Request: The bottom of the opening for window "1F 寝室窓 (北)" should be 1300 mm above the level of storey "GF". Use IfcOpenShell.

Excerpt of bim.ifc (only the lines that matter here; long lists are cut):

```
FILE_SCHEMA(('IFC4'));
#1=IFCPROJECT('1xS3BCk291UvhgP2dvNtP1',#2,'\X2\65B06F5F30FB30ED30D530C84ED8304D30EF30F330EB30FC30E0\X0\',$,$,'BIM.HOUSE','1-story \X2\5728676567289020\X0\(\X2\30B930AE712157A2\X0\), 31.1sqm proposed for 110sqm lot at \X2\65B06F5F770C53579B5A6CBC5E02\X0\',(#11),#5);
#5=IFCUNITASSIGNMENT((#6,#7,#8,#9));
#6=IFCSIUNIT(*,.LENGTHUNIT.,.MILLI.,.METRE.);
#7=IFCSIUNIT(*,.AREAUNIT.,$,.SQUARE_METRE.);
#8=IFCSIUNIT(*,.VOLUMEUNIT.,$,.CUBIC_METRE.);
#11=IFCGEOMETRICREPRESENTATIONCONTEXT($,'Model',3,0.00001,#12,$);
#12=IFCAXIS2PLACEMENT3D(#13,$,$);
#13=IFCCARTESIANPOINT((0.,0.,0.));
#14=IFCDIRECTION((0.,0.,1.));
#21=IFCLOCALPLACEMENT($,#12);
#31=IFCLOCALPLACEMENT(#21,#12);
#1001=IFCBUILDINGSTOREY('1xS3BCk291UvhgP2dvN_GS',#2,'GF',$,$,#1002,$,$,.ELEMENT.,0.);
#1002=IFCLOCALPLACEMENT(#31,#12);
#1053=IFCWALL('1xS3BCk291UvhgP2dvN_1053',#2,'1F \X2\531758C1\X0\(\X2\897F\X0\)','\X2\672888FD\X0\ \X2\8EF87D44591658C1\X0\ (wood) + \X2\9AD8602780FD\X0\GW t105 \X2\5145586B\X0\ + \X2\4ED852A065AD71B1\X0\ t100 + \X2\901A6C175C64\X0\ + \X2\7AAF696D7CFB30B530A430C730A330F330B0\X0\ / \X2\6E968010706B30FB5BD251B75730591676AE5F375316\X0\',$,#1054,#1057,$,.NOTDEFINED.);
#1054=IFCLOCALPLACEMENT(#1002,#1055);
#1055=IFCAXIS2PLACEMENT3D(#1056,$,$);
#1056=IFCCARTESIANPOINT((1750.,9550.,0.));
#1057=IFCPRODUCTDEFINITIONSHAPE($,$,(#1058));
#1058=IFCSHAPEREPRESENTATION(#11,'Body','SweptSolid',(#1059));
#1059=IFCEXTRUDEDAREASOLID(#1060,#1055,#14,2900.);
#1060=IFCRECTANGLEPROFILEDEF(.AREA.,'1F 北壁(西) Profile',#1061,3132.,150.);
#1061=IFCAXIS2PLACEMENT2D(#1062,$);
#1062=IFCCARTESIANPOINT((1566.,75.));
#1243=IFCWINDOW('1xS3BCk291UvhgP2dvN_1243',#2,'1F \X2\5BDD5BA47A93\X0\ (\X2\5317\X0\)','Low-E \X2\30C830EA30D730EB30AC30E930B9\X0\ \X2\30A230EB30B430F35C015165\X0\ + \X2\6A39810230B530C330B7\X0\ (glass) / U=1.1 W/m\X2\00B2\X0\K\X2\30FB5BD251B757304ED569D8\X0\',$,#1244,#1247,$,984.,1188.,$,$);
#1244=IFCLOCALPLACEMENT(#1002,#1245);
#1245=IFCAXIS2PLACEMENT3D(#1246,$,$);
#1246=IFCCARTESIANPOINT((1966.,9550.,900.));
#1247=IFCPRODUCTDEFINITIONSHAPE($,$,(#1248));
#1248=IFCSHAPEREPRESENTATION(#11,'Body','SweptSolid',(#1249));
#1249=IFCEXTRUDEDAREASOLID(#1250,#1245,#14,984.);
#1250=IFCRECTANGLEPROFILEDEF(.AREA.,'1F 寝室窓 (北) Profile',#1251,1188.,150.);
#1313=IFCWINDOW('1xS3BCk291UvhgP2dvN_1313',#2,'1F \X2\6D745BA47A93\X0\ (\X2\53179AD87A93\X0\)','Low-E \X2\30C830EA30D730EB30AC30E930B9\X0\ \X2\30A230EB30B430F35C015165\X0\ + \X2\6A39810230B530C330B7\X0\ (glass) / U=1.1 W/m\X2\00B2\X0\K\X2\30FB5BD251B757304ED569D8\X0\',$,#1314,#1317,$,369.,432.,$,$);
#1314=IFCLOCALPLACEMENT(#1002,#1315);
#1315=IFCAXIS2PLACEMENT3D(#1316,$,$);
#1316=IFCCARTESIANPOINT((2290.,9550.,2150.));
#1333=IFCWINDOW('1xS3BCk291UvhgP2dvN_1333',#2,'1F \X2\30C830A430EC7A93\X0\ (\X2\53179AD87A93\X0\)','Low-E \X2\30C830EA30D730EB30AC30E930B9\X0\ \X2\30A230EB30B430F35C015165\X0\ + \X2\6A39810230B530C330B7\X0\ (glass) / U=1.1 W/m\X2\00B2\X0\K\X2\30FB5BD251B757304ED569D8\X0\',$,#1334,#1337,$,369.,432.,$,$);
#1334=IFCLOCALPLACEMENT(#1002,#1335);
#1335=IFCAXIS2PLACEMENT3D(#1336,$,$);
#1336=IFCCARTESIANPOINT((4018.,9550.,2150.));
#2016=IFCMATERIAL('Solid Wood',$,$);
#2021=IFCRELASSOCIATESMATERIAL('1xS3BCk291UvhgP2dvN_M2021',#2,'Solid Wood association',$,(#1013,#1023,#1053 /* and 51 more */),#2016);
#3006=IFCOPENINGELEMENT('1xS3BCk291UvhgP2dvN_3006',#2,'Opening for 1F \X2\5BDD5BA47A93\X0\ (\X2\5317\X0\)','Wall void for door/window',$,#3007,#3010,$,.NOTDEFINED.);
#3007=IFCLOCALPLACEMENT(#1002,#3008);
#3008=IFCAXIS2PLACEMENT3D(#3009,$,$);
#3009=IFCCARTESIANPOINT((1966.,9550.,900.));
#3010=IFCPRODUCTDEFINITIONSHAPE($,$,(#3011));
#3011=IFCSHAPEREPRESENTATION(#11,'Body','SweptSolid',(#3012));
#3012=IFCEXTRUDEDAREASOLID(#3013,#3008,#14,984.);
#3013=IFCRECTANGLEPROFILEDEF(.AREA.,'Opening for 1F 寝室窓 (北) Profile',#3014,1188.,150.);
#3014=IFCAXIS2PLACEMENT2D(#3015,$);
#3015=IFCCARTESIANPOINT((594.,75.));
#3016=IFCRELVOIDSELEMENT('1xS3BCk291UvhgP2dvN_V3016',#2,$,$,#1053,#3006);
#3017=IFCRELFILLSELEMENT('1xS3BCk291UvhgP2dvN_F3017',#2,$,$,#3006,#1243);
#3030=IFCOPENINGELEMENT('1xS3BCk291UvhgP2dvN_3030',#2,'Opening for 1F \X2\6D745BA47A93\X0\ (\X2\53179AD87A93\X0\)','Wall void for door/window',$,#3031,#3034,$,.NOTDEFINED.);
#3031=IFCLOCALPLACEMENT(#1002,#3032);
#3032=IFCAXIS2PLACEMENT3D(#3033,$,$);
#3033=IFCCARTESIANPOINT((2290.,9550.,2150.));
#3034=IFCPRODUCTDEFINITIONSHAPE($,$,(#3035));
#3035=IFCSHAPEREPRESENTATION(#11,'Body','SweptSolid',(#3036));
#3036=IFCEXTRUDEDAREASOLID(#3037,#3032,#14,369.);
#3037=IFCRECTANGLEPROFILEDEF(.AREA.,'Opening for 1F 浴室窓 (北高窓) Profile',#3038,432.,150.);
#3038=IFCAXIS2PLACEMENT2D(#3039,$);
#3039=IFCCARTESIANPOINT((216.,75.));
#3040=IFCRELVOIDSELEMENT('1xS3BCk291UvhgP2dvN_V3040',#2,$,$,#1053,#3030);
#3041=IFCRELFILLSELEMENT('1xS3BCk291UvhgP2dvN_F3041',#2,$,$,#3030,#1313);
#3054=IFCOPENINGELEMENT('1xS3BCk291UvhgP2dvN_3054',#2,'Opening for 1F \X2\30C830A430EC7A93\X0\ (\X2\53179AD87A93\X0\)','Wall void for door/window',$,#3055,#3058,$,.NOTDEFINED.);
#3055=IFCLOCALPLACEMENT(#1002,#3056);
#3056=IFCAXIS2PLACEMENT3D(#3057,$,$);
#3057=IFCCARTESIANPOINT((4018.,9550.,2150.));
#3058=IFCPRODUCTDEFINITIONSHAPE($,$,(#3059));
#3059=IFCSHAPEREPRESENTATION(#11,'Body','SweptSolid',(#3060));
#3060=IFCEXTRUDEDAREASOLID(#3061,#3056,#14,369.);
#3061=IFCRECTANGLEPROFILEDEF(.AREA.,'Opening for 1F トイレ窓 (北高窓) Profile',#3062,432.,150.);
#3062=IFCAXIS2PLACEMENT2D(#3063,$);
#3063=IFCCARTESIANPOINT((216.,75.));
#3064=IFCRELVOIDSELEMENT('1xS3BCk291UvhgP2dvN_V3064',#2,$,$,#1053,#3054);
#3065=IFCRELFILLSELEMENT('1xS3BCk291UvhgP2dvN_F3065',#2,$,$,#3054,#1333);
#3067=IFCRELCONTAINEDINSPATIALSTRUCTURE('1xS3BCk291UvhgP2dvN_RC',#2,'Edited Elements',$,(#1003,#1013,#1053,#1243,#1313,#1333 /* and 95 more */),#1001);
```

```python
import numpy as np
import ifcopenshell
import ifcopenshell.api.geometry
import ifcopenshell.geom
import ifcopenshell.util.element
import ifcopenshell.util.placement
import ifcopenshell.util.shape
import ifcopenshell.util.unit

model = ifcopenshell.open("bim.ifc")
unit_scale = ifcopenshell.util.unit.calculate_unit_scale(model)

window = model.by_guid("1xS3BCk291UvhgP2dvN_1243")
opening = window.FillsVoids[0].RelatingOpeningElement
storey = ifcopenshell.util.element.get_container(window, ifc_class="IfcBuildingStorey")
level = ifcopenshell.util.placement.get_local_placement(storey.ObjectPlacement)[2, 3]

# The opening's origin need not be at the sill, so measure its lowest point.
shape = ifcopenshell.geom.create_shape(ifcopenshell.geom.settings(), opening)
bottom = ifcopenshell.util.shape.get_shape_bottom_elevation(shape, shape.geometry) / unit_scale
dz = level + 1300.0 - bottom

shift = np.array([0.0, 0.0, dz])
# The window is not placed relative to its opening, so move both.
for product in (opening, window):
    matrix = ifcopenshell.util.placement.get_local_placement(product.ObjectPlacement)
    matrix[:3, 3] += shift
    ifcopenshell.api.geometry.edit_object_placement(model, product=product, matrix=matrix, is_si=False)

print(f"moved by {dz * unit_scale:+.3f} m")

model.write("bim_v2.ifc")
```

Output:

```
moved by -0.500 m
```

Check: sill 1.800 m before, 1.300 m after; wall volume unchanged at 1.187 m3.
